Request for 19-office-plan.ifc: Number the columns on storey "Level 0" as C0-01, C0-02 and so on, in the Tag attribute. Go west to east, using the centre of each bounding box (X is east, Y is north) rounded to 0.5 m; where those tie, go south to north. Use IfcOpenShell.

First a look at what the model holds.

```python
import ifcopenshell
import ifcopenshell.util.element
import ifcopenshell.util.placement

model = ifcopenshell.open("19-office-plan.ifc")
print(model.schema)
storey = next(s for s in model.by_type("IfcBuildingStorey") if s.Name == "Level 0")
columns = [e for e in ifcopenshell.util.element.get_decomposition(storey) if e.is_a("IfcColumn")]
for e in sorted(columns, key=lambda e: e.id()):
    origin = ifcopenshell.util.placement.get_local_placement(e.ObjectPlacement)[:3, 3]
    print(e.id(), e.Tag, e.Name, origin.round(2) + 0.0, sep=" | ")
```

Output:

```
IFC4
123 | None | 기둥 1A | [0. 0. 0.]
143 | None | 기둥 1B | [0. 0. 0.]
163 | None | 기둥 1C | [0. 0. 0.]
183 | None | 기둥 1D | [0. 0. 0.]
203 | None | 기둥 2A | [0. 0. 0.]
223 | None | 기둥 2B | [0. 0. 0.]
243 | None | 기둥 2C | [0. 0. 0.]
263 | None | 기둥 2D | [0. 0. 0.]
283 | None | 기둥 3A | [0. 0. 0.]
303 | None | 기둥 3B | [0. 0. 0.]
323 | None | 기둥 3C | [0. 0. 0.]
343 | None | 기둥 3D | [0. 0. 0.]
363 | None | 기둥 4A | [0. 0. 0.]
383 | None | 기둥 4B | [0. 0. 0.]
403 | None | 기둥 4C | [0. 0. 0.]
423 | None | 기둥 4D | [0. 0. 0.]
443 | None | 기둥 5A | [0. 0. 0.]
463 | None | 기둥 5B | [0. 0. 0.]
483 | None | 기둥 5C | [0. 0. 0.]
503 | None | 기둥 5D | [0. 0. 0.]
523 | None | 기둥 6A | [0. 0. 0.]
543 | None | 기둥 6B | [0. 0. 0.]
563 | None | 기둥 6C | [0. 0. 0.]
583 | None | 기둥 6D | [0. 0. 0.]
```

```python
import ifcopenshell
import ifcopenshell.geom
import ifcopenshell.util.element
import ifcopenshell.util.shape

model = ifcopenshell.open("19-office-plan.ifc")
settings = ifcopenshell.geom.settings()
settings.set("use-world-coords", True)


def centre(element):
    shape = ifcopenshell.geom.create_shape(settings, element)
    return ifcopenshell.util.shape.get_bbox_centroid(shape.geometry)


storey = next(s for s in model.by_type("IfcBuildingStorey") if s.Name == "Level 0")
columns = [e for e in ifcopenshell.util.element.get_decomposition(storey) if e.is_a("IfcColumn")]

# Insertion points can sit at a corner or the storey origin, so sort by the geometry (in metres).
centres = {e: centre(e) for e in columns}
columns.sort(key=lambda e: (round(centres[e][0] / 0.5), centres[e][1]))

for i, e in enumerate(columns, start=1):
    number = f"C0-{i:02d}"
    e.Tag = number
    print(e.id(), number)

model.write("19-office-plan-out.ifc")
```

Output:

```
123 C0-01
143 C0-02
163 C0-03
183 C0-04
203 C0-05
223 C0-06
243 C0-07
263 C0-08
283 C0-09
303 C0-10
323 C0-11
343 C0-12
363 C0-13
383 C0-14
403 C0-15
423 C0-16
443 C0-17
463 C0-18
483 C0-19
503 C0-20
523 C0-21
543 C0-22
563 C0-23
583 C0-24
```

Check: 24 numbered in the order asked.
